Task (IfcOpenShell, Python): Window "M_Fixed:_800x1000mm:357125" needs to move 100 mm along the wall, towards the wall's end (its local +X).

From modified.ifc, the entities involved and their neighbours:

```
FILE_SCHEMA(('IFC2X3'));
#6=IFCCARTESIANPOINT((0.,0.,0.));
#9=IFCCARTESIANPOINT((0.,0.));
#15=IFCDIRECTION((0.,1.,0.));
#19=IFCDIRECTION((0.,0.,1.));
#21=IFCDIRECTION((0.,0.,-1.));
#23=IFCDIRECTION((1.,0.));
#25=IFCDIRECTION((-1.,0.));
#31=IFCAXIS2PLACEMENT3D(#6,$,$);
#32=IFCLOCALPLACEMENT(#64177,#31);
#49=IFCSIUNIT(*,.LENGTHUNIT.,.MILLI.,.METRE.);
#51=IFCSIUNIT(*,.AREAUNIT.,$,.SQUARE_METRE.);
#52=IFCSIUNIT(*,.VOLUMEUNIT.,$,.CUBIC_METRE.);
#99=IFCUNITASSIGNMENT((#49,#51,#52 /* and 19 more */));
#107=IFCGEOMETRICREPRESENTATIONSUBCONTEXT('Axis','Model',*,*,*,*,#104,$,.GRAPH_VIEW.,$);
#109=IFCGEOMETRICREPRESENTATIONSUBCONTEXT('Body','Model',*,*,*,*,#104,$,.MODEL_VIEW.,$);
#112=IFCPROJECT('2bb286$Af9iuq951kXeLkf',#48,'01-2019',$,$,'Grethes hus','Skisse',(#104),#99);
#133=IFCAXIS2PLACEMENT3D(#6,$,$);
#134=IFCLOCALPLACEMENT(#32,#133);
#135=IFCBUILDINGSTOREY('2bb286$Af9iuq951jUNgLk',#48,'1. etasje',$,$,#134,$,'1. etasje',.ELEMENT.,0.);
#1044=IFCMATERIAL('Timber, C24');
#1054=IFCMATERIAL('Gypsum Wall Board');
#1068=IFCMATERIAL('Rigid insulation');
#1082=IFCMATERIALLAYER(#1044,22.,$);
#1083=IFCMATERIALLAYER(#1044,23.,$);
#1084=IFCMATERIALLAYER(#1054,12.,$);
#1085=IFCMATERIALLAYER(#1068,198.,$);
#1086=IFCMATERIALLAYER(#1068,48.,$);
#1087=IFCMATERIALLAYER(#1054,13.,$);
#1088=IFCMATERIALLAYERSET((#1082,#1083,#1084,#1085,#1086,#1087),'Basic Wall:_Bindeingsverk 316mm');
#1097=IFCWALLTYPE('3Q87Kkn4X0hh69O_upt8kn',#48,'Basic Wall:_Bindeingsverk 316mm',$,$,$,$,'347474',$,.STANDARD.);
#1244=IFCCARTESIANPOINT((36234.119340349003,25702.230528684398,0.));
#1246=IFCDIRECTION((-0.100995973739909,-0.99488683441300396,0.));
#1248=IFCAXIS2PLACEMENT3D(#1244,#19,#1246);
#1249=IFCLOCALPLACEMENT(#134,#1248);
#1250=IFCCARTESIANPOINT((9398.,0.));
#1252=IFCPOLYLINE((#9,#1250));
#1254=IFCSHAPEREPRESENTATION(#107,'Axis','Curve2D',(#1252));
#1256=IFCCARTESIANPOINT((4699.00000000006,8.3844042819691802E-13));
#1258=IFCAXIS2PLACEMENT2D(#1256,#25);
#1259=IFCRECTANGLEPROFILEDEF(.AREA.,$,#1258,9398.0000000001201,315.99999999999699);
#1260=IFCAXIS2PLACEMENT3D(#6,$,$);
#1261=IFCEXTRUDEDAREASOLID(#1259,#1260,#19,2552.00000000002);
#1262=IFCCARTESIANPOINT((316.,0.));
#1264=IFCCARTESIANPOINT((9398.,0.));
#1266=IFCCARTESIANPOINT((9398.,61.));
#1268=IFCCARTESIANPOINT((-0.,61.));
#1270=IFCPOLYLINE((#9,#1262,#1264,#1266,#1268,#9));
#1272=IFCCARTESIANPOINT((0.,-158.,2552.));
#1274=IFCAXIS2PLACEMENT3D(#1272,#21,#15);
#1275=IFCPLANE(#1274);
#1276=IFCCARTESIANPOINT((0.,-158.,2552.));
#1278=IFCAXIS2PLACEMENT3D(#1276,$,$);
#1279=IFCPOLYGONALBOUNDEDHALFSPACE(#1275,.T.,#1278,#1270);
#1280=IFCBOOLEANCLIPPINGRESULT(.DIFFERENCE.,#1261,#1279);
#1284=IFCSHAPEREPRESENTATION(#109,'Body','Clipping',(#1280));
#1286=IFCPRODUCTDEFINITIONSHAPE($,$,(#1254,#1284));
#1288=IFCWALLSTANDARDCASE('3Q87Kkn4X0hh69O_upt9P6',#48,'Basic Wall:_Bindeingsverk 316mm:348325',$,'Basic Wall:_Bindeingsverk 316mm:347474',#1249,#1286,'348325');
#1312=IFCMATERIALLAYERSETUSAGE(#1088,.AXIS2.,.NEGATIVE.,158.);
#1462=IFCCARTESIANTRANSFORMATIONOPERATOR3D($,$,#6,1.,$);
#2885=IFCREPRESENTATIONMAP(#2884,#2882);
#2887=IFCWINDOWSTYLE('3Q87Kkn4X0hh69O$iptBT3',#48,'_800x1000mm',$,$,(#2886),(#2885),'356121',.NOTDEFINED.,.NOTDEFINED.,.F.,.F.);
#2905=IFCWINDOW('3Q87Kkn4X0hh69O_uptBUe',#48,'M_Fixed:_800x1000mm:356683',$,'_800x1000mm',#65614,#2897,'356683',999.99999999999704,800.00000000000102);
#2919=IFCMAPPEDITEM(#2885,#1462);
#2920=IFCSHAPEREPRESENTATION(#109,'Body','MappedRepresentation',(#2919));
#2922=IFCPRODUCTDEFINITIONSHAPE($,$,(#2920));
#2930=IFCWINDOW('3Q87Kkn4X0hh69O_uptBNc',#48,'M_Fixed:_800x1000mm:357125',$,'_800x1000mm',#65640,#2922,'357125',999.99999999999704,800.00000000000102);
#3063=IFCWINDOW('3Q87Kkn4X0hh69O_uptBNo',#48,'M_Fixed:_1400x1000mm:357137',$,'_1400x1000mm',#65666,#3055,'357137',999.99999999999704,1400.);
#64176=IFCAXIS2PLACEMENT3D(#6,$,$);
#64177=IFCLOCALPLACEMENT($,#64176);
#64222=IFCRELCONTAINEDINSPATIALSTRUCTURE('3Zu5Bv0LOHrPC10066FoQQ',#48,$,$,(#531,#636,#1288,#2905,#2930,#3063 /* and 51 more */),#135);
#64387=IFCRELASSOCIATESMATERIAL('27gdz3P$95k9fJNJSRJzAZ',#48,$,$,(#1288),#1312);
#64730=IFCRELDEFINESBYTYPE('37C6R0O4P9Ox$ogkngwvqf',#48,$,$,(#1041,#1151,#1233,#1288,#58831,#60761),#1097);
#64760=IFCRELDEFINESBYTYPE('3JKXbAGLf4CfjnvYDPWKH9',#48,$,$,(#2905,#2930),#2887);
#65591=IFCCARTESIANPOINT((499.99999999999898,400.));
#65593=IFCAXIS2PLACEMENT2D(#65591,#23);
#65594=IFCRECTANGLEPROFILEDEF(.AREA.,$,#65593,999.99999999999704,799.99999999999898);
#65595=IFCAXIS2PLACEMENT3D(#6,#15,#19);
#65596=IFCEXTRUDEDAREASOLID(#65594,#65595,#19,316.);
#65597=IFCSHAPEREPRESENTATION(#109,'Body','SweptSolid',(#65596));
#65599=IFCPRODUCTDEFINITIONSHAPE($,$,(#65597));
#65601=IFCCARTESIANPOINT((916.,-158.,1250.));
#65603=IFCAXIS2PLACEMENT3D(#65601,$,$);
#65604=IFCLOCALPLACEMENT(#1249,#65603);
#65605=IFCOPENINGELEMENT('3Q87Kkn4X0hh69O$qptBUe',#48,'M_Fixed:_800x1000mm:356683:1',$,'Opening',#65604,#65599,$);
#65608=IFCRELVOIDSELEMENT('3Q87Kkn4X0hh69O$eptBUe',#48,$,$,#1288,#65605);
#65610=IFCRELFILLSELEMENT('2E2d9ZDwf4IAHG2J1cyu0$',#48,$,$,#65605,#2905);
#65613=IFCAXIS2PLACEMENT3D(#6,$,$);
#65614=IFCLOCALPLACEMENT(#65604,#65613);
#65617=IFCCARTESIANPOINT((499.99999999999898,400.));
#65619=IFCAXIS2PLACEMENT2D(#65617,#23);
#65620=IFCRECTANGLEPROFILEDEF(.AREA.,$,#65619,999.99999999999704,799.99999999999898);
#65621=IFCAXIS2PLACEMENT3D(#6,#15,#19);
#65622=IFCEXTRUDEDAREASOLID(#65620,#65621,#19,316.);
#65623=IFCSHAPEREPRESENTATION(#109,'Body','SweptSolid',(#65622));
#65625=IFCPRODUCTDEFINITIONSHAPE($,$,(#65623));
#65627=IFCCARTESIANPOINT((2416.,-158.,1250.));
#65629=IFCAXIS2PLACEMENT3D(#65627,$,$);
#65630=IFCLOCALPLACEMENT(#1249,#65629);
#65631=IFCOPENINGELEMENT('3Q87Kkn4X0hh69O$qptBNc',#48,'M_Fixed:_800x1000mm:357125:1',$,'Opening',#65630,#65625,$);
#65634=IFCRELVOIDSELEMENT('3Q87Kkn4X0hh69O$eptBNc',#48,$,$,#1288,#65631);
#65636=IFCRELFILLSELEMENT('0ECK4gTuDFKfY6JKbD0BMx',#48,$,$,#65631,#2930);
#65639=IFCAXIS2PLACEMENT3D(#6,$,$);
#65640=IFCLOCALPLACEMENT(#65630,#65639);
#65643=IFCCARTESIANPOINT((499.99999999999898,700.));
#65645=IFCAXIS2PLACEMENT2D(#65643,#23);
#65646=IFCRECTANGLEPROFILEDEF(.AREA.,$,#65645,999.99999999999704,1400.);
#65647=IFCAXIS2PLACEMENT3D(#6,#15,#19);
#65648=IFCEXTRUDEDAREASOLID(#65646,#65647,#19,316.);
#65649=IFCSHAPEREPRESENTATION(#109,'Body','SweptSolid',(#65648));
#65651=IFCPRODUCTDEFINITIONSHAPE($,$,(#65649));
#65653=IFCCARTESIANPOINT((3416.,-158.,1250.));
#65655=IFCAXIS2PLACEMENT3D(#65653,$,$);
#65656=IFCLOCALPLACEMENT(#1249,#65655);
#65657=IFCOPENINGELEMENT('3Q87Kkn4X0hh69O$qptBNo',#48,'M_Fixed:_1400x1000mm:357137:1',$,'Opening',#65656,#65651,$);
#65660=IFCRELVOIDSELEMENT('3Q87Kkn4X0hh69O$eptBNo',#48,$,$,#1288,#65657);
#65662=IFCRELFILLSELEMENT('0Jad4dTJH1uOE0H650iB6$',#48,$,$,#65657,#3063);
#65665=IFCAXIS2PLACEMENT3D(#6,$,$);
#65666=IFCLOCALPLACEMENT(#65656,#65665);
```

```python
import ifcopenshell
import ifcopenshell.api.geometry
import ifcopenshell.util.placement

model = ifcopenshell.open("modified.ifc")

window = model.by_guid("3Q87Kkn4X0hh69O_uptBNc")
opening = window.FillsVoids[0].RelatingOpeningElement
wall = opening.VoidsElements[0].RelatingBuildingElement

wall_matrix = ifcopenshell.util.placement.get_local_placement(wall.ObjectPlacement)
shift = wall_matrix[:3, 0] * 100.0
before = ifcopenshell.util.placement.get_local_placement(window.ObjectPlacement)[:3, 3].copy()

# The window is placed relative to its opening, so it follows when the opening moves.
matrix = ifcopenshell.util.placement.get_local_placement(opening.ObjectPlacement)
matrix[:3, 3] += shift
ifcopenshell.api.geometry.edit_object_placement(
    model, product=opening, matrix=matrix, is_si=False, should_transform_children=True
)

after = ifcopenshell.util.placement.get_local_placement(window.ObjectPlacement)[:3, 3]
print("window moved by", (after - before).round(3) + 0.0)

model.write("modified_updated.ifc")
```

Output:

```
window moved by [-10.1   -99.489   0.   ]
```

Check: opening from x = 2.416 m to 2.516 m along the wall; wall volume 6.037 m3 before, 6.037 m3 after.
